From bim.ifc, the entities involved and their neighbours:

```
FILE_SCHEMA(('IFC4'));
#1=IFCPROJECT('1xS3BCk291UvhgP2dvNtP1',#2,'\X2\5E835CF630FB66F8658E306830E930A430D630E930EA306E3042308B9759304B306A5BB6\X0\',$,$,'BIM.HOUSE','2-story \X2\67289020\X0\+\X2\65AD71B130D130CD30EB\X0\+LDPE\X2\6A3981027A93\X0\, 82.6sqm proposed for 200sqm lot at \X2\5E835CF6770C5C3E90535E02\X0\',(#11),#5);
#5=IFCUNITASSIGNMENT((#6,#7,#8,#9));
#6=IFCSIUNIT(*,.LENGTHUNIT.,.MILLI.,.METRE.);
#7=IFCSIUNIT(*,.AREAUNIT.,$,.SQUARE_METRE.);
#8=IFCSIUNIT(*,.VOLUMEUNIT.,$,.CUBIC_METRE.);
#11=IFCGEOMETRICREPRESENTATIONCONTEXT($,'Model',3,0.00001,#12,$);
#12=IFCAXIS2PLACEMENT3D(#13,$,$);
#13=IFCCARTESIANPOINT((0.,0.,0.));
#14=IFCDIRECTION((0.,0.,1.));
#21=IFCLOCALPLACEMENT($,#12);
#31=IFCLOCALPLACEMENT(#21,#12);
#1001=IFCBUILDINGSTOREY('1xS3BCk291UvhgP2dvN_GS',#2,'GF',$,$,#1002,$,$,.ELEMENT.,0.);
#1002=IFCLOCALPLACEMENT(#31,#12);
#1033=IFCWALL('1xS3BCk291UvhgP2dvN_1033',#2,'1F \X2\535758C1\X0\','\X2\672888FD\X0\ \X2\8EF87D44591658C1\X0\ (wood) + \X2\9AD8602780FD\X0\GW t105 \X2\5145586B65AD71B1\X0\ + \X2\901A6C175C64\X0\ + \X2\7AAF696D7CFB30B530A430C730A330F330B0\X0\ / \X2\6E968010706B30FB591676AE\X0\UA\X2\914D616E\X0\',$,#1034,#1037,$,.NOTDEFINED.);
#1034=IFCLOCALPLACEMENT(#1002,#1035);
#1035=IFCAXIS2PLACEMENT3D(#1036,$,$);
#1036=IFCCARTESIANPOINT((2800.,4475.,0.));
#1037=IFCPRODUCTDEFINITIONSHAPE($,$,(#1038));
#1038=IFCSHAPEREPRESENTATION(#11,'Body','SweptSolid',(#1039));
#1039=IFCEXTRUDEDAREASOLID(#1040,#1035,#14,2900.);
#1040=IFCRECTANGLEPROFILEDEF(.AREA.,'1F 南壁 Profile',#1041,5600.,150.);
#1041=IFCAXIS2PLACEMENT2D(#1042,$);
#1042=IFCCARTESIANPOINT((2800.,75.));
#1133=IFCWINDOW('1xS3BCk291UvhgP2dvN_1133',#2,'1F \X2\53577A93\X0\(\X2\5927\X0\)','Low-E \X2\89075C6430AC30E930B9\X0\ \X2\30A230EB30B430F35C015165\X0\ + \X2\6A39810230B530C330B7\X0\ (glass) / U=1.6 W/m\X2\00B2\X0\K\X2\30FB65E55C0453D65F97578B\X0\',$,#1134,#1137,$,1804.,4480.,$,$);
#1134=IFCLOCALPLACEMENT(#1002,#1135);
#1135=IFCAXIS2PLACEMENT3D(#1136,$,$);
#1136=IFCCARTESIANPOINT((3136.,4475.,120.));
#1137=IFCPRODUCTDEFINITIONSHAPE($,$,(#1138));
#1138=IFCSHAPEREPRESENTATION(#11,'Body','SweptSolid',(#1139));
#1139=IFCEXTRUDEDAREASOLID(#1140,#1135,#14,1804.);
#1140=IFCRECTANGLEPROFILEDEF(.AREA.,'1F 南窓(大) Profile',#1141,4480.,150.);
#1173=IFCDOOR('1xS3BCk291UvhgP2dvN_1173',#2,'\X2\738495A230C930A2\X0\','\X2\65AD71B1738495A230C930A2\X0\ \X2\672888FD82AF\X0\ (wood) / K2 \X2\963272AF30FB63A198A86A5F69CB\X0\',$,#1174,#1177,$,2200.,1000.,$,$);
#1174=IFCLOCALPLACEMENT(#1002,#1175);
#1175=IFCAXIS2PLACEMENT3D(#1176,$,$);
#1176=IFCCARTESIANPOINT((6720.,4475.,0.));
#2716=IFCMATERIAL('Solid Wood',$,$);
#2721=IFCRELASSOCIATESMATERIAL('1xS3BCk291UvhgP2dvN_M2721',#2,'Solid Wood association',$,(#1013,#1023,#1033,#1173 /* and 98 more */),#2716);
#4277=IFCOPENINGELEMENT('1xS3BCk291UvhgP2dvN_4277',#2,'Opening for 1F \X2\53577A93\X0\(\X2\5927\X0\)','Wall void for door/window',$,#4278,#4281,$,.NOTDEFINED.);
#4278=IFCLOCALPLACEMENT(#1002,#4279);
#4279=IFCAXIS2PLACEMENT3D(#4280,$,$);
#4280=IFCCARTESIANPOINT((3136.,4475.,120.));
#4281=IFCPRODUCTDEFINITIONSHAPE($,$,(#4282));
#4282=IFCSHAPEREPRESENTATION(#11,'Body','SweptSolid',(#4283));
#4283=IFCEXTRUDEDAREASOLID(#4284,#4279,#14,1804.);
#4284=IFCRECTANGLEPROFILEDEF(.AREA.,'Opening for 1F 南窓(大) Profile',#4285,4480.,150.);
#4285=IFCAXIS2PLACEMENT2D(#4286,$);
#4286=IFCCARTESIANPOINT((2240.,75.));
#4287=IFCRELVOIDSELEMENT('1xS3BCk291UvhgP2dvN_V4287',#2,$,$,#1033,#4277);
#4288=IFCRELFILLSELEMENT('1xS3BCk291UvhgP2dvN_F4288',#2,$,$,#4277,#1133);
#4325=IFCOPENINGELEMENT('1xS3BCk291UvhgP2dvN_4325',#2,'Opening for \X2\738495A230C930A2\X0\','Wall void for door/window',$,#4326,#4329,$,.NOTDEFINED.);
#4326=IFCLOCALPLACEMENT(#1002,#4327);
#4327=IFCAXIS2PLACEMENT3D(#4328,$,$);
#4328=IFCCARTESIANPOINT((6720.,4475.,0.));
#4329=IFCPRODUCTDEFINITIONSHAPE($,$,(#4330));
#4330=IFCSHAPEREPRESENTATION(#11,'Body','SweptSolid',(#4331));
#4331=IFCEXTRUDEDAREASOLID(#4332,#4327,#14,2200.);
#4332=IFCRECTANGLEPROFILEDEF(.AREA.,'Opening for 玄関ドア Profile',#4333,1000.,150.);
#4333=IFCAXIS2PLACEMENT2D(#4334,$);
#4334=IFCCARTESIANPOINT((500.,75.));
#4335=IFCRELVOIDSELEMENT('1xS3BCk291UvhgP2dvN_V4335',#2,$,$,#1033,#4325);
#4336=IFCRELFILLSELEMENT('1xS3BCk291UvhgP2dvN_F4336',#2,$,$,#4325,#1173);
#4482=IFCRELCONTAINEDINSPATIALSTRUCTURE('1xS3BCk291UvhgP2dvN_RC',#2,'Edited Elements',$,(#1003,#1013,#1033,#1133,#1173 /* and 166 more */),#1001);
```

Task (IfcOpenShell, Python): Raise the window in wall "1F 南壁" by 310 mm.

```python
import numpy as np
import ifcopenshell
import ifcopenshell.api.geometry
import ifcopenshell.util.placement
import ifcopenshell.util.unit

model = ifcopenshell.open("bim.ifc")
unit_scale = ifcopenshell.util.unit.calculate_unit_scale(model)

window = model.by_id(1133)
opening = window.FillsVoids[0].RelatingOpeningElement
dz = 0.31 / unit_scale

shift = np.array([0.0, 0.0, dz])
# The window is not placed relative to its opening, so move both.
for product in (opening, window):
    matrix = ifcopenshell.util.placement.get_local_placement(product.ObjectPlacement)
    matrix[:3, 3] += shift
    ifcopenshell.api.geometry.edit_object_placement(model, product=product, matrix=matrix, is_si=False)

print(f"moved by {dz * unit_scale:+.3f} m")

model.write("bim_edited.ifc")
```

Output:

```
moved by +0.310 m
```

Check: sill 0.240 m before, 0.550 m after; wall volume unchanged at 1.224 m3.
